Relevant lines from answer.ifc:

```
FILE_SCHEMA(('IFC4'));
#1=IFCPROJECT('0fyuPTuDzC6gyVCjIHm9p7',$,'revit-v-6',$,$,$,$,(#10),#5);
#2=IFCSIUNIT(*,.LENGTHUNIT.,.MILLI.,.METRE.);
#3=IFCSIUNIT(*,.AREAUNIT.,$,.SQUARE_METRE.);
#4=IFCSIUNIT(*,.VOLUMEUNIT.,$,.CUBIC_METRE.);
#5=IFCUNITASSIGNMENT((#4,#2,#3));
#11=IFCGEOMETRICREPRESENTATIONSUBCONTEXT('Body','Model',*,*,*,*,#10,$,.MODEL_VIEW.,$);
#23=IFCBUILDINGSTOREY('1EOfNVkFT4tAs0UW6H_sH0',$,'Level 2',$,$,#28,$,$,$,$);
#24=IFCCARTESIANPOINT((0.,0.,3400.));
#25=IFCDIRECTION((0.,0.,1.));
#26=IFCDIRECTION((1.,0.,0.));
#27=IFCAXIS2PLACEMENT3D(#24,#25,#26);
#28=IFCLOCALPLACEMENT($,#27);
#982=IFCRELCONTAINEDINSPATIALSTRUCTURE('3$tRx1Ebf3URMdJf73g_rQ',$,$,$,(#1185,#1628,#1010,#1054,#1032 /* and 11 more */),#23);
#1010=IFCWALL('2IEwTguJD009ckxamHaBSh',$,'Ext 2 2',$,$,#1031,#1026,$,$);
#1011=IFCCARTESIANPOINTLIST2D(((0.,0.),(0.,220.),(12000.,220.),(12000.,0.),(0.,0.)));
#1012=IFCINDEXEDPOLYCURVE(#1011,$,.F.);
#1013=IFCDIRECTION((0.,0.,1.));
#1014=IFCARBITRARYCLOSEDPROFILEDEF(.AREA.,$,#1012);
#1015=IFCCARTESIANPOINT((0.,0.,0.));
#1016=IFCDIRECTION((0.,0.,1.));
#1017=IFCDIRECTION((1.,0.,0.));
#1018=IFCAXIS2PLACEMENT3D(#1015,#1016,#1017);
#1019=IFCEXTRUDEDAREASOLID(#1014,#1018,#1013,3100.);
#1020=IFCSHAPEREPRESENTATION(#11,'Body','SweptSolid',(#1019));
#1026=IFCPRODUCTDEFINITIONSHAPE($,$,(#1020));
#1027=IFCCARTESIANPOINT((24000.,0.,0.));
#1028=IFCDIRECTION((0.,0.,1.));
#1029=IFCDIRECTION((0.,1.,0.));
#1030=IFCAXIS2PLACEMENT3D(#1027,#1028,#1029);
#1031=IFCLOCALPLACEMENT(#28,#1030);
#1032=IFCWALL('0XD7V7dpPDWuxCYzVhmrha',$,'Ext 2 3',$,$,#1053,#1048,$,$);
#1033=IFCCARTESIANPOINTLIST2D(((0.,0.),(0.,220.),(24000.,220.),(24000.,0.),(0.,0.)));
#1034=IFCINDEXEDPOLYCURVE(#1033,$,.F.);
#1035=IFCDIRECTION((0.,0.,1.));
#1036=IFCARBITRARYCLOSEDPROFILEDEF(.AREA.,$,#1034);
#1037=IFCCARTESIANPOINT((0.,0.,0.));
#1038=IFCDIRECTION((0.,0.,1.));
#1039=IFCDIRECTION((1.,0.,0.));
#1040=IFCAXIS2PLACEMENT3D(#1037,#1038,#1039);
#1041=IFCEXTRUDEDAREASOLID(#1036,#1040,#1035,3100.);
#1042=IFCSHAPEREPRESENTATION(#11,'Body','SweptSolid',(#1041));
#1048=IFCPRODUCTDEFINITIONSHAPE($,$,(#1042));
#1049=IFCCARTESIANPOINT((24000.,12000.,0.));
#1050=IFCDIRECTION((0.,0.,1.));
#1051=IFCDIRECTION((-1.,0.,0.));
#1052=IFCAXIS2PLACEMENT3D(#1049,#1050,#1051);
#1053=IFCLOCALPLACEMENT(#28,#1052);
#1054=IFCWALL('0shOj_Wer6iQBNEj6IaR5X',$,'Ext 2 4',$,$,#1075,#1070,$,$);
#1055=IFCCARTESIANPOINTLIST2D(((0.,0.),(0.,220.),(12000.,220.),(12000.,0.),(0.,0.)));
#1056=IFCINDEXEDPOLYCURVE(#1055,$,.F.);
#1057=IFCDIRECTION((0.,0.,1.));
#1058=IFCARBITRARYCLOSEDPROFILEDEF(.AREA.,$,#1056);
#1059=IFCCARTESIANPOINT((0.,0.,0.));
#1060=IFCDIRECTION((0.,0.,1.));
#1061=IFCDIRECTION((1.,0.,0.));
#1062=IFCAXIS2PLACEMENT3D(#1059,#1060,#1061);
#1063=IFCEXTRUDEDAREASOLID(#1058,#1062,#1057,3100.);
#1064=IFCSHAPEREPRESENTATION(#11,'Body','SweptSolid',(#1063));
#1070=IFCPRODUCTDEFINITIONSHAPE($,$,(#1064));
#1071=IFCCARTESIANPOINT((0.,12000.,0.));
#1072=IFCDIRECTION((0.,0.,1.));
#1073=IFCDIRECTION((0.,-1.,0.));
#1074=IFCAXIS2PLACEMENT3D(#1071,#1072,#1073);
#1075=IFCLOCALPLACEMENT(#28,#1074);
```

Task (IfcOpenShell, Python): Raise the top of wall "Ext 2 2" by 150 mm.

```python
import ifcopenshell
import ifcopenshell.geom
import ifcopenshell.util.representation
import ifcopenshell.util.shape

model = ifcopenshell.open("answer.ifc")
settings = ifcopenshell.geom.settings()


def volume(element):
    """Net volume in cubic metres, openings subtracted."""
    shape = ifcopenshell.geom.create_shape(settings, element)
    return ifcopenshell.util.shape.get_volume(shape.geometry)


wall = model.by_guid("2IEwTguJD009ckxamHaBSh")
before = volume(wall)

body = ifcopenshell.util.representation.get_representation(wall, "Model", "Body")
solid = body.Items[0]
old_height = solid.Depth
solid.Depth += 150.0
after = volume(wall)

print(f"height {old_height:g} -> {solid.Depth:g}, volume {before:.3f} -> {after:.3f} m3")

model.write("answer-out.ifc")
```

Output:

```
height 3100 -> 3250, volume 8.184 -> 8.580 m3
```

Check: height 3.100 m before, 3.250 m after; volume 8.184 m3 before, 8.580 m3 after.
